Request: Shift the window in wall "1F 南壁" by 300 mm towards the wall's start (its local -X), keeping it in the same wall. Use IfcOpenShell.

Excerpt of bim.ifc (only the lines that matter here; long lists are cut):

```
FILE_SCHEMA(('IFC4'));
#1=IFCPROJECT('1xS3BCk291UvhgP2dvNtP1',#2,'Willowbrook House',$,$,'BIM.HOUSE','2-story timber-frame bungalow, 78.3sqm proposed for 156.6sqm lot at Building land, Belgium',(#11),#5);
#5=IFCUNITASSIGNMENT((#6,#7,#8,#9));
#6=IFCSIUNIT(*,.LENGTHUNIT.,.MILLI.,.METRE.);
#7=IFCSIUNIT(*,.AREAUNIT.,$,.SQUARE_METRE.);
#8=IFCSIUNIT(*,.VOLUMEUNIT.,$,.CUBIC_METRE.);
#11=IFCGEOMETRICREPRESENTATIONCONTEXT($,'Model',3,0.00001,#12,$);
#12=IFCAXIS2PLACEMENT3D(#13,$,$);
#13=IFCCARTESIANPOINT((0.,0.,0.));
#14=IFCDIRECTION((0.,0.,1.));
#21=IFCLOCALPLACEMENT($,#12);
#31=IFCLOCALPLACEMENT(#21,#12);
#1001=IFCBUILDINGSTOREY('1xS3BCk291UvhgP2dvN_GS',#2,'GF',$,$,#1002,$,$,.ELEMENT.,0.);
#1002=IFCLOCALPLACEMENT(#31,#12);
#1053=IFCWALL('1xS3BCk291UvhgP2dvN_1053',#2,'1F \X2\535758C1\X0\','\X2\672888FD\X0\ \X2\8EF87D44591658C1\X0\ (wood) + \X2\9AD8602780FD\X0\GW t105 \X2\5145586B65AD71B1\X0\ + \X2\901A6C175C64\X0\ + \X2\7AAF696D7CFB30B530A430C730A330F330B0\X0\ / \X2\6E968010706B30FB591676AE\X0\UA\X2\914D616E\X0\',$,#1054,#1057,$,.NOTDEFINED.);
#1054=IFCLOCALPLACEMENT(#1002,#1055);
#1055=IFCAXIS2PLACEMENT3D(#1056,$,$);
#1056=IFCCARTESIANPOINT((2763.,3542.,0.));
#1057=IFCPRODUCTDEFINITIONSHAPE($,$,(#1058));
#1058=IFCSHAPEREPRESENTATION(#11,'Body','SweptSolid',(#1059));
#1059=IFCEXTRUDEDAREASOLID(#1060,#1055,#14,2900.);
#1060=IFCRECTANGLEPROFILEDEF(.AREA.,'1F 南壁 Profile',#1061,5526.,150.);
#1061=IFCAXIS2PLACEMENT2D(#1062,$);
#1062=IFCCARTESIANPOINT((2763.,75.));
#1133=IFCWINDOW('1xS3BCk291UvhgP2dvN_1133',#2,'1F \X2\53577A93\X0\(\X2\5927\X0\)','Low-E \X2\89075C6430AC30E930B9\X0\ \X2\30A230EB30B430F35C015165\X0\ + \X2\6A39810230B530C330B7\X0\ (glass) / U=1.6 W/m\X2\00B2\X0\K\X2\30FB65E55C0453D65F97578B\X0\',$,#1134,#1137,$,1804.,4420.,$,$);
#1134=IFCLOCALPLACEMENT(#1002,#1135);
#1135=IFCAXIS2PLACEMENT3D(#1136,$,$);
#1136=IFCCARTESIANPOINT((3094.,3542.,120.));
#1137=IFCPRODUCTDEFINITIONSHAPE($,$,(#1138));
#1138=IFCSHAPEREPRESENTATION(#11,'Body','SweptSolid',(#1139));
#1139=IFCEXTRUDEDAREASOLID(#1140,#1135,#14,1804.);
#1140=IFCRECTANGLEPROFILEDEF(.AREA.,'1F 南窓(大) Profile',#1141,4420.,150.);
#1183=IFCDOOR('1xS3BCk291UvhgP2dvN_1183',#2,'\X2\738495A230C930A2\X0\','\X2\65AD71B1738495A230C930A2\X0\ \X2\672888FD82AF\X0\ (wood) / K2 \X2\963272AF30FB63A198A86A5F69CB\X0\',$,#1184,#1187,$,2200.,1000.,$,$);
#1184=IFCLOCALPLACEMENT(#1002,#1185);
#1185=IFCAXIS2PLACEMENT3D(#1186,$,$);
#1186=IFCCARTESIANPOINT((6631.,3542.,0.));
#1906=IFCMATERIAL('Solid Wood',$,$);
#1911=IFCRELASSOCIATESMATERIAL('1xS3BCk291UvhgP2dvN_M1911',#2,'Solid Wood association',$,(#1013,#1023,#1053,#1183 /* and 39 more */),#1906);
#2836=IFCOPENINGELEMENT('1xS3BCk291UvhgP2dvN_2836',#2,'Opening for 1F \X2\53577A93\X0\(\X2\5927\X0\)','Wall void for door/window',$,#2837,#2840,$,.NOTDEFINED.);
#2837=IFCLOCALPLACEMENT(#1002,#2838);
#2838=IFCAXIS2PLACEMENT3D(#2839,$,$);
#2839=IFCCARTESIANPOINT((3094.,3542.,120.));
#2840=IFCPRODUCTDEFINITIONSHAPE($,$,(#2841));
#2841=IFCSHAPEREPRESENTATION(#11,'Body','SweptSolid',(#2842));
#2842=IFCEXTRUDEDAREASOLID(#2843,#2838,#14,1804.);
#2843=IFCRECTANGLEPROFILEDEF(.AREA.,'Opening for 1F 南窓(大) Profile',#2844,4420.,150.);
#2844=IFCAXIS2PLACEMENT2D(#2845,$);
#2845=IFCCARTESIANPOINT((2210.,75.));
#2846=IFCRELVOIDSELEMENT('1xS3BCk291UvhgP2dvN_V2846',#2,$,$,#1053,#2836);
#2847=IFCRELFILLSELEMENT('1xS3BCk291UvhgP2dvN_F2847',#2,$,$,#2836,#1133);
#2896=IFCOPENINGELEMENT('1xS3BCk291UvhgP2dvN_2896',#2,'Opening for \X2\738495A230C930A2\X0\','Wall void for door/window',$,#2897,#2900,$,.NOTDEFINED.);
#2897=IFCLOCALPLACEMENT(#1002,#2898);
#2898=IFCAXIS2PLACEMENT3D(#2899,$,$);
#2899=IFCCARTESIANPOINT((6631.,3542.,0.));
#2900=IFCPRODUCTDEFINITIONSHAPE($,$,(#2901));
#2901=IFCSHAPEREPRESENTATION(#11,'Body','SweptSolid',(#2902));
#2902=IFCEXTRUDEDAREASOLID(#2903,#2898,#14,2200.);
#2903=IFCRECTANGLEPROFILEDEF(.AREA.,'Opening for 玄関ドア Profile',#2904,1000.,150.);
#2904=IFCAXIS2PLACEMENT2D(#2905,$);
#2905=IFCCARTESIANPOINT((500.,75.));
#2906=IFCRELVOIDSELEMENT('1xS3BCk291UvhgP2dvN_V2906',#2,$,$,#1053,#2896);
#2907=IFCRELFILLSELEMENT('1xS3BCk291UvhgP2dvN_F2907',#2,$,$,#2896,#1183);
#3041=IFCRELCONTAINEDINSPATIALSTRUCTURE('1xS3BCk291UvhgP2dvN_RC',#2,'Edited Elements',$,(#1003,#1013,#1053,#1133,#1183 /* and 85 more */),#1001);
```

```python
import ifcopenshell
import ifcopenshell.api.geometry
import ifcopenshell.util.placement
import ifcopenshell.util.unit

model = ifcopenshell.open("bim.ifc")
unit_scale = ifcopenshell.util.unit.calculate_unit_scale(model)

window = model.by_guid("1xS3BCk291UvhgP2dvN_1133")
opening = window.FillsVoids[0].RelatingOpeningElement
wall = opening.VoidsElements[0].RelatingBuildingElement

wall_matrix = ifcopenshell.util.placement.get_local_placement(wall.ObjectPlacement)
shift = wall_matrix[:3, 0] * -0.3 / unit_scale
before = ifcopenshell.util.placement.get_local_placement(window.ObjectPlacement)[:3, 3].copy()

# The window is not placed relative to its opening, so move both.
for product in (opening, window):
    matrix = ifcopenshell.util.placement.get_local_placement(product.ObjectPlacement)
    matrix[:3, 3] += shift
    ifcopenshell.api.geometry.edit_object_placement(model, product=product, matrix=matrix, is_si=False)

after = ifcopenshell.util.placement.get_local_placement(window.ObjectPlacement)[:3, 3]
print("window moved by", (after - before).round(3) + 0.0)

model.write("bim_edited.ifc")
```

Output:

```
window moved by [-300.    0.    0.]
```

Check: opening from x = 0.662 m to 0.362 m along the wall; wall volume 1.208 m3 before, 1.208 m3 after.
